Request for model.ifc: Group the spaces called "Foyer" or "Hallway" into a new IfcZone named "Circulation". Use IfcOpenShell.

First a look at what the model holds.

```python
import ifcopenshell

model = ifcopenshell.open("model.ifc")
print(model.schema)
seen = {}
for space in model.by_type("IfcSpace"):
    seen[space.LongName] = seen.get(space.LongName, 0) + 1
for name, count in sorted(seen.items(), key=str):
    print(count, "x", name)
print("zones:", [z.Name for z in model.by_type("IfcZone")][:20])
```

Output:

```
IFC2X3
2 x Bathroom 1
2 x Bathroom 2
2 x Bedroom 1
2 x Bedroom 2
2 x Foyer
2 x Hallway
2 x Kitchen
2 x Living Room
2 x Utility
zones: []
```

```python
import ifcopenshell
import ifcopenshell.api.group
import ifcopenshell.api.root

model = ifcopenshell.open("model.ifc")

names = {"Foyer", "Hallway"}
spaces = [s for s in model.by_type("IfcSpace") if s.LongName in names]

zone = ifcopenshell.api.root.create_entity(model, ifc_class="IfcZone", name="Circulation")
ifcopenshell.api.group.assign_group(model, products=spaces, group=zone)
print(len(spaces), "spaces in", zone.Name)

model.write("model_v2.ifc")
```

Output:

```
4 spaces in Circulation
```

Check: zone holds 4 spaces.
